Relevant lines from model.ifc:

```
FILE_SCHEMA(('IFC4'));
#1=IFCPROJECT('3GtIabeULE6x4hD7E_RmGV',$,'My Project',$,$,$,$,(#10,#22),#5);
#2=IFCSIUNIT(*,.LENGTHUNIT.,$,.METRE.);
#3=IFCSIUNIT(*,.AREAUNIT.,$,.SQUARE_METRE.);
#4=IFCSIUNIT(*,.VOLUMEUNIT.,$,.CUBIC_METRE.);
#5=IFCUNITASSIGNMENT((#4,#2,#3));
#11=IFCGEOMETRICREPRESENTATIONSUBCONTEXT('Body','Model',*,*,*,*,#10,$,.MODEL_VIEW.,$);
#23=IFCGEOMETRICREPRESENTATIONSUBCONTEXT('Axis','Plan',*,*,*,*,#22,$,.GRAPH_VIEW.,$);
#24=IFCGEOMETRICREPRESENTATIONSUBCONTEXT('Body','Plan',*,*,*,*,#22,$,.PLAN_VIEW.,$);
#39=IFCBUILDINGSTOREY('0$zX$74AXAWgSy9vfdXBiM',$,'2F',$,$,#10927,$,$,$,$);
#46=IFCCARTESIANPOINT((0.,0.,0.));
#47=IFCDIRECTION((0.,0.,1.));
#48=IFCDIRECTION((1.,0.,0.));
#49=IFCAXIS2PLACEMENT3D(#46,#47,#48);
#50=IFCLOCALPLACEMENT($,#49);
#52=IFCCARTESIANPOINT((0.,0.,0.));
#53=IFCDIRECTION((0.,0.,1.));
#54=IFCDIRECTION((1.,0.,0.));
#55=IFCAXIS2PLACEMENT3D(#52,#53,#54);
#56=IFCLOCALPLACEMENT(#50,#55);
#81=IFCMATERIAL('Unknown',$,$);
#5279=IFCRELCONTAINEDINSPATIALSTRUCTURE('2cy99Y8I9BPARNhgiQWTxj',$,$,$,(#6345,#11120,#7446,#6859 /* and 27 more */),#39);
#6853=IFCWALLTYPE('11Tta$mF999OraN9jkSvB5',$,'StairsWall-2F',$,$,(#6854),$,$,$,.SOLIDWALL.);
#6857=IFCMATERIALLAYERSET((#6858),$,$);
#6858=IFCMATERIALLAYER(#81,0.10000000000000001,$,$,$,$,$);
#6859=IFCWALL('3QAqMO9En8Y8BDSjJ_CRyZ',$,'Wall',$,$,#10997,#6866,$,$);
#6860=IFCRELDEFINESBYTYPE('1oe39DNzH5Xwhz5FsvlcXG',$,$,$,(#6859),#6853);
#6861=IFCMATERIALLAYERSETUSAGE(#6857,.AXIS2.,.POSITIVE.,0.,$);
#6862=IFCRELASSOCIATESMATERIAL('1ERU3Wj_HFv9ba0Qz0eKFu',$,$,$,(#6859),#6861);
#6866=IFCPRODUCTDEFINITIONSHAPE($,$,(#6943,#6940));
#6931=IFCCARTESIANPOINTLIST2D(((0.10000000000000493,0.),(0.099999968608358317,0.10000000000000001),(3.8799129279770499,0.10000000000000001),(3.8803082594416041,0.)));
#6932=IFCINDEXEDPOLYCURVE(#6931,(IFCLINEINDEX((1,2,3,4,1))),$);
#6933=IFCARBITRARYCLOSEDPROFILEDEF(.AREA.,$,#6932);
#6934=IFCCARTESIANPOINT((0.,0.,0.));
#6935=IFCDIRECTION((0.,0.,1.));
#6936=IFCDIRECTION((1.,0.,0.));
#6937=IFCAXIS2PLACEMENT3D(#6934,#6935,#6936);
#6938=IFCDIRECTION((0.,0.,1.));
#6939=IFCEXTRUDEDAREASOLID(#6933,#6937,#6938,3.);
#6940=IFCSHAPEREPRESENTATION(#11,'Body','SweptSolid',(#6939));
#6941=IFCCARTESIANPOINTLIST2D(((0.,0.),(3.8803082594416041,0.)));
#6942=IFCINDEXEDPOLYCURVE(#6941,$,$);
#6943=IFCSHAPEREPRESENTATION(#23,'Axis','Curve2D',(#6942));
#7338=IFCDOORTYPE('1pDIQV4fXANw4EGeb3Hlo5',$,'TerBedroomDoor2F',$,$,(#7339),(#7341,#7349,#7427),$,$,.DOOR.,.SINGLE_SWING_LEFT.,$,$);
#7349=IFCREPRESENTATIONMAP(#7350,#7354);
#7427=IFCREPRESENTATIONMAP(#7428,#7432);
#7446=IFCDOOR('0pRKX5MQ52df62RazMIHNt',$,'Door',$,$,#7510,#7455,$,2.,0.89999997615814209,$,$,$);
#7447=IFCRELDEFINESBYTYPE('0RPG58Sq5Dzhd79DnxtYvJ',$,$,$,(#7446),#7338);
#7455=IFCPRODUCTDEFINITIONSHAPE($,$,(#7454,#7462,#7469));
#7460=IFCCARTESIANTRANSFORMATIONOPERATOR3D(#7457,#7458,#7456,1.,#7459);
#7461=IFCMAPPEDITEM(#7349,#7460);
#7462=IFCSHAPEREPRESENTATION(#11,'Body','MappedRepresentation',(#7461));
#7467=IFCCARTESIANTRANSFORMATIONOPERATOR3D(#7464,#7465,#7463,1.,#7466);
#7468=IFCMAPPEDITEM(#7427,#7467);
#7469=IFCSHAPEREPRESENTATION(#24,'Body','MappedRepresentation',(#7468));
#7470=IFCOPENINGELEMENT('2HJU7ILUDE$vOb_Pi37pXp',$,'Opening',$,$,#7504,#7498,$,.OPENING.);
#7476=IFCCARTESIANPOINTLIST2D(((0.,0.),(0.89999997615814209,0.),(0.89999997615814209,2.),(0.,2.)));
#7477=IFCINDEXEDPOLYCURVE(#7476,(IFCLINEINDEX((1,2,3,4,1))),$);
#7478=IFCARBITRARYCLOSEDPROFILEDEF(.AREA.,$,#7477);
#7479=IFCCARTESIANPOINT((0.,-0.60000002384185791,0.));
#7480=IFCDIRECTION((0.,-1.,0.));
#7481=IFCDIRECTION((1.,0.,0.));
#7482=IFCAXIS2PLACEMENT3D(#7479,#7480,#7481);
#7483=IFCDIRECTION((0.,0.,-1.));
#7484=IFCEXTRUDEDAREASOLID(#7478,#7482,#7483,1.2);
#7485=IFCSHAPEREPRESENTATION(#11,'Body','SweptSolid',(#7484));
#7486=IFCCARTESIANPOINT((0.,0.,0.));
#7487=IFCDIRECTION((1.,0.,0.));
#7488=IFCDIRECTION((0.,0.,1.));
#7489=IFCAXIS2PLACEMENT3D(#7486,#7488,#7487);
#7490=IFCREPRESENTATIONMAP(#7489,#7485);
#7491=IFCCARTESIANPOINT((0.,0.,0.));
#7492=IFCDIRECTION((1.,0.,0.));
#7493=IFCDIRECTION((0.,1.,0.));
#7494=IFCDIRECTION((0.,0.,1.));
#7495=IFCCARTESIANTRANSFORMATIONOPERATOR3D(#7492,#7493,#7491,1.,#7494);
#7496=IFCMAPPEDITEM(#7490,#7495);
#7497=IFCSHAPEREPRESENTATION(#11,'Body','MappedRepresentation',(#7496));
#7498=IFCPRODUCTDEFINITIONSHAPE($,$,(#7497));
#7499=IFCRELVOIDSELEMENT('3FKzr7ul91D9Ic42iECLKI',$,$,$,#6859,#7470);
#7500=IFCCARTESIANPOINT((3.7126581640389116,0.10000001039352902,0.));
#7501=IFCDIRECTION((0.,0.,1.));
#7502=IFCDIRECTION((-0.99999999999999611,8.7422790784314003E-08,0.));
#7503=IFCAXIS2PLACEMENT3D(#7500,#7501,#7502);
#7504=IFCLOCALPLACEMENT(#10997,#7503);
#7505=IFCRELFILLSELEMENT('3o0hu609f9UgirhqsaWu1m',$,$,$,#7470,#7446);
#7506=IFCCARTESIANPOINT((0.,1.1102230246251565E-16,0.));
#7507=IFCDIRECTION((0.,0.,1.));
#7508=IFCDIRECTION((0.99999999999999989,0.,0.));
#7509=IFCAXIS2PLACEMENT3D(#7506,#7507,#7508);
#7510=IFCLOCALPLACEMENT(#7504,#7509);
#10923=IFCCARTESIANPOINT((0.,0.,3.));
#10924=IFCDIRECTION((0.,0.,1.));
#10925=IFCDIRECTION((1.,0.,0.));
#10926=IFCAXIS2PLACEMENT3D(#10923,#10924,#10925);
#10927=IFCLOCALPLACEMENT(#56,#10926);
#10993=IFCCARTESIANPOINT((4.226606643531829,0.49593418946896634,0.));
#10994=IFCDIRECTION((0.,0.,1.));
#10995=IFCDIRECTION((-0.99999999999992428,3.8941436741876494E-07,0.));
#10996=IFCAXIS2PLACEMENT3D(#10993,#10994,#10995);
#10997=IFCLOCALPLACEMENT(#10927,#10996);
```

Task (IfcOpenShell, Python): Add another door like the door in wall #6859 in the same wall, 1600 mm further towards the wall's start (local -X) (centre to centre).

```python
import ifcopenshell
import ifcopenshell.api.feature
import ifcopenshell.api.geometry
import ifcopenshell.api.root
import ifcopenshell.geom
import ifcopenshell.util.element
import ifcopenshell.util.placement
import ifcopenshell.util.shape
import ifcopenshell.util.unit

model = ifcopenshell.open("model.ifc")
unit_scale = ifcopenshell.util.unit.calculate_unit_scale(model)
settings = ifcopenshell.geom.settings()


def volume(element):
    """Net volume in cubic metres, openings subtracted."""
    shape = ifcopenshell.geom.create_shape(settings, element)
    return ifcopenshell.util.shape.get_volume(shape.geometry)


door = model.by_guid("0pRKX5MQ52df62RazMIHNt")
opening = door.FillsVoids[0].RelatingOpeningElement
wall = opening.VoidsElements[0].RelatingBuildingElement
before = volume(wall)
shift = ifcopenshell.util.placement.get_local_placement(wall.ObjectPlacement)[:3, 0] * -1.6 / unit_scale

# copy_class copies the void relationship, type, container and properties, but no geometry.
new_opening = ifcopenshell.api.root.copy_class(model, product=opening)
new_opening.Representation = ifcopenshell.util.element.copy_deep(
    model, opening.Representation, exclude=["IfcGeometricRepresentationContext", "IfcRepresentationMap"]
)
new_door = ifcopenshell.api.root.copy_class(model, product=door)
new_door.Representation = ifcopenshell.util.element.copy_deep(
    model, door.Representation, exclude=["IfcGeometricRepresentationContext", "IfcRepresentationMap"]
)
ifcopenshell.api.feature.add_filling(model, opening=new_opening, element=new_door)

for old, new in ((opening, new_opening), (door, new_door)):
    matrix = ifcopenshell.util.placement.get_local_placement(old.ObjectPlacement)
    matrix[:3, 3] += shift
    ifcopenshell.api.geometry.edit_object_placement(model, product=new, matrix=matrix, is_si=False)

after = volume(wall)

print(f"wall volume {before:.3f} -> {after:.3f} m3")

model.write("model_edited.ifc")
```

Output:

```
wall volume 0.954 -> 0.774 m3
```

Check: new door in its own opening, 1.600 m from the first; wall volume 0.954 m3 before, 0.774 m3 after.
